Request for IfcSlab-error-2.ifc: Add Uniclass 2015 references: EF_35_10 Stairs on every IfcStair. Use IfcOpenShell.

First a look at what the model holds.

```python
import ifcopenshell

model = ifcopenshell.open("IfcSlab-error-2.ifc")
print(model.schema)
print("classifications:", [c.Name for c in model.by_type("IfcClassification")])
for ifc_class in ("IfcDoor", "IfcRoof", "IfcStair", "IfcWall", "IfcWindow"):
    print(ifc_class, len(model.by_type(ifc_class)))
```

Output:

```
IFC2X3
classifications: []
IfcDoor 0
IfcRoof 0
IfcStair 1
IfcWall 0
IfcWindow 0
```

```python
import ifcopenshell
import ifcopenshell.api.classification

model = ifcopenshell.open("IfcSlab-error-2.ifc")

# IFC2X3 requires Source and Edition and has no link from the project to the system.
system = model.create_entity("IfcClassification", Source="NBS", Edition="2015", Name="Uniclass 2015")

codes = {
    "IfcStair": ("EF_35_10", "Stairs"),
}
for ifc_class, (code, name) in codes.items():
    products = model.by_type(ifc_class)
    ifcopenshell.api.classification.add_reference(
        model, products=products, classification=system, identification=code, name=name
    )
    print(code, len(products))

model.write("IfcSlab-error-2_edited.ifc")
```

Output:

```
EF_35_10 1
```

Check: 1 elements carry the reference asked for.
